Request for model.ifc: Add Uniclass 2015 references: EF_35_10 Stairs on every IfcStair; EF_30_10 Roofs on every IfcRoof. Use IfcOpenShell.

First a look at what the model holds.

```python
import ifcopenshell

model = ifcopenshell.open("model.ifc")
print(model.schema)
print("classifications:", [c.Name for c in model.by_type("IfcClassification")])
for ifc_class in ("IfcDoor", "IfcRoof", "IfcStair", "IfcWall", "IfcWindow"):
    print(ifc_class, len(model.by_type(ifc_class)))
```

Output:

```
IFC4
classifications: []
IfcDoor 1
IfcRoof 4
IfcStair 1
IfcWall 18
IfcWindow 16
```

```python
import ifcopenshell
import ifcopenshell.api.classification

model = ifcopenshell.open("model.ifc")

system = ifcopenshell.api.classification.add_classification(model, classification="Uniclass 2015")

codes = {
    "IfcStair": ("EF_35_10", "Stairs"),
    "IfcRoof": ("EF_30_10", "Roofs"),
}
for ifc_class, (code, name) in codes.items():
    products = model.by_type(ifc_class)
    ifcopenshell.api.classification.add_reference(
        model, products=products, classification=system, identification=code, name=name
    )
    print(code, len(products))

model.write("model_edited.ifc")
```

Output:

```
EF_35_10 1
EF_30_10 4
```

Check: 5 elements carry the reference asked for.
